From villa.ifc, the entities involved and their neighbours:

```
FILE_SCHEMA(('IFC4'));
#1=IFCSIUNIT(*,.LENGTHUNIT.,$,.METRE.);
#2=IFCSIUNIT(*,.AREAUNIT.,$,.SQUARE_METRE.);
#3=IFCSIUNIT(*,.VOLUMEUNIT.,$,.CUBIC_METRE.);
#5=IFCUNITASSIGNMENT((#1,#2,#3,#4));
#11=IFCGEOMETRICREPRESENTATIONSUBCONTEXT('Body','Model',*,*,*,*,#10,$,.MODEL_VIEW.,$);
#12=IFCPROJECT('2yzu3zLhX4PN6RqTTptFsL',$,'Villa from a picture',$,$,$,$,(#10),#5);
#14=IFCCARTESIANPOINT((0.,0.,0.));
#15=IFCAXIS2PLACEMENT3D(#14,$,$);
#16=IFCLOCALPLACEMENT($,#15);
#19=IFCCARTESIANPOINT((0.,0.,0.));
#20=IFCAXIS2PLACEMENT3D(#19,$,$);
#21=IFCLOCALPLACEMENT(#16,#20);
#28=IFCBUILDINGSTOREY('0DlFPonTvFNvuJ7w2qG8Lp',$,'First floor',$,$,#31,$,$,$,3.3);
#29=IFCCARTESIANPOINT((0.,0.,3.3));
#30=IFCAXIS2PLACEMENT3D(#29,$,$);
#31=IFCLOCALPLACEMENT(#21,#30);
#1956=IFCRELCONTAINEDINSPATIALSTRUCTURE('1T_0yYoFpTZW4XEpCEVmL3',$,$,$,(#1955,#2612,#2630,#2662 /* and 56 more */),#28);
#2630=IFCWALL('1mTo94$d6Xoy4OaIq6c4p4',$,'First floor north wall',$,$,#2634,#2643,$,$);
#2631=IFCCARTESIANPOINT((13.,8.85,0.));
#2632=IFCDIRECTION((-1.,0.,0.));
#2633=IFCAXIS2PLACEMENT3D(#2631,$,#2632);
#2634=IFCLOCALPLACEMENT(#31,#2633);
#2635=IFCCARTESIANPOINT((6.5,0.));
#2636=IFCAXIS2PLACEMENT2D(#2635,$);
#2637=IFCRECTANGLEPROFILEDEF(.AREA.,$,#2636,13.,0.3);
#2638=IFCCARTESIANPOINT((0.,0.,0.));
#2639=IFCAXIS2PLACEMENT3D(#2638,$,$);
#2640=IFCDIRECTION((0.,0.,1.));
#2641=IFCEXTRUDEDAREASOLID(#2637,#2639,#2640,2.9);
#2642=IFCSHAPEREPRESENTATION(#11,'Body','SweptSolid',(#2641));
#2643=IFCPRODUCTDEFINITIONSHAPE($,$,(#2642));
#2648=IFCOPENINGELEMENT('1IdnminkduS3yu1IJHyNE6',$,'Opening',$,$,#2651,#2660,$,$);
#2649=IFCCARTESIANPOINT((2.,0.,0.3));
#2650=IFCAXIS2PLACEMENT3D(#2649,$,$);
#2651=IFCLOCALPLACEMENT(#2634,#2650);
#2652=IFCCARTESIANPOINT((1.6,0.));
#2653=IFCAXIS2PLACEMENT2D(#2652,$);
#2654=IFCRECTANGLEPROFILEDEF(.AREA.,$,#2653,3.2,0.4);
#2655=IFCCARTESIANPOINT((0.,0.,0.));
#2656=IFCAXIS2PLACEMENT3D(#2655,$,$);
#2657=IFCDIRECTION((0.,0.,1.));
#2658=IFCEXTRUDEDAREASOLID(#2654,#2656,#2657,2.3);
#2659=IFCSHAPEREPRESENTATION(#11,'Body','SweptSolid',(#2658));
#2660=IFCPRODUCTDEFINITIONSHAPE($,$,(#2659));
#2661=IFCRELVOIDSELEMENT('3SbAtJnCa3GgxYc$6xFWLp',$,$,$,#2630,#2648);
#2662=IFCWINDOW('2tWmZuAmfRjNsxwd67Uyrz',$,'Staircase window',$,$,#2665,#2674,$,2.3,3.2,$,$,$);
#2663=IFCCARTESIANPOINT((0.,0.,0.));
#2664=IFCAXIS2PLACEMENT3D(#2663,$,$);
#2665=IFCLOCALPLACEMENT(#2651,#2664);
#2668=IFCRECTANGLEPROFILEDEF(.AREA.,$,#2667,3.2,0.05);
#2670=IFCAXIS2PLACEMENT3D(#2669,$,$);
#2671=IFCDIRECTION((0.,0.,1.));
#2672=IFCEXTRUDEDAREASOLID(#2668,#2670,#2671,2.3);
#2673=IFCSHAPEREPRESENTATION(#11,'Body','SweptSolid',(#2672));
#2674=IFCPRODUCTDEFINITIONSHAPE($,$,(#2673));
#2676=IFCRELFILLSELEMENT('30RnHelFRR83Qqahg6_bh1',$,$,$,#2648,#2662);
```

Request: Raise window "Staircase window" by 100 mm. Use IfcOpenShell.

```python
import numpy as np
import ifcopenshell
import ifcopenshell.api.geometry
import ifcopenshell.util.placement
import ifcopenshell.util.unit

model = ifcopenshell.open("villa.ifc")
unit_scale = ifcopenshell.util.unit.calculate_unit_scale(model)

window = model.by_id(2662)
opening = window.FillsVoids[0].RelatingOpeningElement
dz = 0.1

shift = np.array([0.0, 0.0, dz])
# The window is placed relative to its opening, so it follows when the opening moves.
matrix = ifcopenshell.util.placement.get_local_placement(opening.ObjectPlacement)
matrix[:3, 3] += shift
ifcopenshell.api.geometry.edit_object_placement(
    model, product=opening, matrix=matrix, is_si=False, should_transform_children=True
)

print(f"moved by {dz * unit_scale:+.3f} m")

model.write("villa_v2.ifc")
```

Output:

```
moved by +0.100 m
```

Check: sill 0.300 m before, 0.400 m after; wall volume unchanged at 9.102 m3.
